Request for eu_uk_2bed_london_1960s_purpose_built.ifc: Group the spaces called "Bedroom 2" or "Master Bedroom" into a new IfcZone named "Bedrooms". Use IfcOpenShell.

First a look at what the model holds.

```python
import ifcopenshell

model = ifcopenshell.open("eu_uk_2bed_london_1960s_purpose_built.ifc")
print(model.schema)
seen = {}
for space in model.by_type("IfcSpace"):
    seen[space.LongName] = seen.get(space.LongName, 0) + 1
for name, count in sorted(seen.items(), key=str):
    print(count, "x", name)
print("zones:", [z.Name for z in model.by_type("IfcZone")][:20])
```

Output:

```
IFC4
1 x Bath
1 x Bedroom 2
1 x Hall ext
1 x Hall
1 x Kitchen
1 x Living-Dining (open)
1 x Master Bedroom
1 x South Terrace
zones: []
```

```python
import ifcopenshell
import ifcopenshell.api.group
import ifcopenshell.api.root

model = ifcopenshell.open("eu_uk_2bed_london_1960s_purpose_built.ifc")

names = {"Bedroom 2", "Master Bedroom"}
spaces = [s for s in model.by_type("IfcSpace") if s.LongName in names]

zone = ifcopenshell.api.root.create_entity(model, ifc_class="IfcZone", name="Bedrooms")
ifcopenshell.api.group.assign_group(model, products=spaces, group=zone)
print(len(spaces), "spaces in", zone.Name)

model.write("eu_uk_2bed_london_1960s_purpose_built_edited.ifc")
```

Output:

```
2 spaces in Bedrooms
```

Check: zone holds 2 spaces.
